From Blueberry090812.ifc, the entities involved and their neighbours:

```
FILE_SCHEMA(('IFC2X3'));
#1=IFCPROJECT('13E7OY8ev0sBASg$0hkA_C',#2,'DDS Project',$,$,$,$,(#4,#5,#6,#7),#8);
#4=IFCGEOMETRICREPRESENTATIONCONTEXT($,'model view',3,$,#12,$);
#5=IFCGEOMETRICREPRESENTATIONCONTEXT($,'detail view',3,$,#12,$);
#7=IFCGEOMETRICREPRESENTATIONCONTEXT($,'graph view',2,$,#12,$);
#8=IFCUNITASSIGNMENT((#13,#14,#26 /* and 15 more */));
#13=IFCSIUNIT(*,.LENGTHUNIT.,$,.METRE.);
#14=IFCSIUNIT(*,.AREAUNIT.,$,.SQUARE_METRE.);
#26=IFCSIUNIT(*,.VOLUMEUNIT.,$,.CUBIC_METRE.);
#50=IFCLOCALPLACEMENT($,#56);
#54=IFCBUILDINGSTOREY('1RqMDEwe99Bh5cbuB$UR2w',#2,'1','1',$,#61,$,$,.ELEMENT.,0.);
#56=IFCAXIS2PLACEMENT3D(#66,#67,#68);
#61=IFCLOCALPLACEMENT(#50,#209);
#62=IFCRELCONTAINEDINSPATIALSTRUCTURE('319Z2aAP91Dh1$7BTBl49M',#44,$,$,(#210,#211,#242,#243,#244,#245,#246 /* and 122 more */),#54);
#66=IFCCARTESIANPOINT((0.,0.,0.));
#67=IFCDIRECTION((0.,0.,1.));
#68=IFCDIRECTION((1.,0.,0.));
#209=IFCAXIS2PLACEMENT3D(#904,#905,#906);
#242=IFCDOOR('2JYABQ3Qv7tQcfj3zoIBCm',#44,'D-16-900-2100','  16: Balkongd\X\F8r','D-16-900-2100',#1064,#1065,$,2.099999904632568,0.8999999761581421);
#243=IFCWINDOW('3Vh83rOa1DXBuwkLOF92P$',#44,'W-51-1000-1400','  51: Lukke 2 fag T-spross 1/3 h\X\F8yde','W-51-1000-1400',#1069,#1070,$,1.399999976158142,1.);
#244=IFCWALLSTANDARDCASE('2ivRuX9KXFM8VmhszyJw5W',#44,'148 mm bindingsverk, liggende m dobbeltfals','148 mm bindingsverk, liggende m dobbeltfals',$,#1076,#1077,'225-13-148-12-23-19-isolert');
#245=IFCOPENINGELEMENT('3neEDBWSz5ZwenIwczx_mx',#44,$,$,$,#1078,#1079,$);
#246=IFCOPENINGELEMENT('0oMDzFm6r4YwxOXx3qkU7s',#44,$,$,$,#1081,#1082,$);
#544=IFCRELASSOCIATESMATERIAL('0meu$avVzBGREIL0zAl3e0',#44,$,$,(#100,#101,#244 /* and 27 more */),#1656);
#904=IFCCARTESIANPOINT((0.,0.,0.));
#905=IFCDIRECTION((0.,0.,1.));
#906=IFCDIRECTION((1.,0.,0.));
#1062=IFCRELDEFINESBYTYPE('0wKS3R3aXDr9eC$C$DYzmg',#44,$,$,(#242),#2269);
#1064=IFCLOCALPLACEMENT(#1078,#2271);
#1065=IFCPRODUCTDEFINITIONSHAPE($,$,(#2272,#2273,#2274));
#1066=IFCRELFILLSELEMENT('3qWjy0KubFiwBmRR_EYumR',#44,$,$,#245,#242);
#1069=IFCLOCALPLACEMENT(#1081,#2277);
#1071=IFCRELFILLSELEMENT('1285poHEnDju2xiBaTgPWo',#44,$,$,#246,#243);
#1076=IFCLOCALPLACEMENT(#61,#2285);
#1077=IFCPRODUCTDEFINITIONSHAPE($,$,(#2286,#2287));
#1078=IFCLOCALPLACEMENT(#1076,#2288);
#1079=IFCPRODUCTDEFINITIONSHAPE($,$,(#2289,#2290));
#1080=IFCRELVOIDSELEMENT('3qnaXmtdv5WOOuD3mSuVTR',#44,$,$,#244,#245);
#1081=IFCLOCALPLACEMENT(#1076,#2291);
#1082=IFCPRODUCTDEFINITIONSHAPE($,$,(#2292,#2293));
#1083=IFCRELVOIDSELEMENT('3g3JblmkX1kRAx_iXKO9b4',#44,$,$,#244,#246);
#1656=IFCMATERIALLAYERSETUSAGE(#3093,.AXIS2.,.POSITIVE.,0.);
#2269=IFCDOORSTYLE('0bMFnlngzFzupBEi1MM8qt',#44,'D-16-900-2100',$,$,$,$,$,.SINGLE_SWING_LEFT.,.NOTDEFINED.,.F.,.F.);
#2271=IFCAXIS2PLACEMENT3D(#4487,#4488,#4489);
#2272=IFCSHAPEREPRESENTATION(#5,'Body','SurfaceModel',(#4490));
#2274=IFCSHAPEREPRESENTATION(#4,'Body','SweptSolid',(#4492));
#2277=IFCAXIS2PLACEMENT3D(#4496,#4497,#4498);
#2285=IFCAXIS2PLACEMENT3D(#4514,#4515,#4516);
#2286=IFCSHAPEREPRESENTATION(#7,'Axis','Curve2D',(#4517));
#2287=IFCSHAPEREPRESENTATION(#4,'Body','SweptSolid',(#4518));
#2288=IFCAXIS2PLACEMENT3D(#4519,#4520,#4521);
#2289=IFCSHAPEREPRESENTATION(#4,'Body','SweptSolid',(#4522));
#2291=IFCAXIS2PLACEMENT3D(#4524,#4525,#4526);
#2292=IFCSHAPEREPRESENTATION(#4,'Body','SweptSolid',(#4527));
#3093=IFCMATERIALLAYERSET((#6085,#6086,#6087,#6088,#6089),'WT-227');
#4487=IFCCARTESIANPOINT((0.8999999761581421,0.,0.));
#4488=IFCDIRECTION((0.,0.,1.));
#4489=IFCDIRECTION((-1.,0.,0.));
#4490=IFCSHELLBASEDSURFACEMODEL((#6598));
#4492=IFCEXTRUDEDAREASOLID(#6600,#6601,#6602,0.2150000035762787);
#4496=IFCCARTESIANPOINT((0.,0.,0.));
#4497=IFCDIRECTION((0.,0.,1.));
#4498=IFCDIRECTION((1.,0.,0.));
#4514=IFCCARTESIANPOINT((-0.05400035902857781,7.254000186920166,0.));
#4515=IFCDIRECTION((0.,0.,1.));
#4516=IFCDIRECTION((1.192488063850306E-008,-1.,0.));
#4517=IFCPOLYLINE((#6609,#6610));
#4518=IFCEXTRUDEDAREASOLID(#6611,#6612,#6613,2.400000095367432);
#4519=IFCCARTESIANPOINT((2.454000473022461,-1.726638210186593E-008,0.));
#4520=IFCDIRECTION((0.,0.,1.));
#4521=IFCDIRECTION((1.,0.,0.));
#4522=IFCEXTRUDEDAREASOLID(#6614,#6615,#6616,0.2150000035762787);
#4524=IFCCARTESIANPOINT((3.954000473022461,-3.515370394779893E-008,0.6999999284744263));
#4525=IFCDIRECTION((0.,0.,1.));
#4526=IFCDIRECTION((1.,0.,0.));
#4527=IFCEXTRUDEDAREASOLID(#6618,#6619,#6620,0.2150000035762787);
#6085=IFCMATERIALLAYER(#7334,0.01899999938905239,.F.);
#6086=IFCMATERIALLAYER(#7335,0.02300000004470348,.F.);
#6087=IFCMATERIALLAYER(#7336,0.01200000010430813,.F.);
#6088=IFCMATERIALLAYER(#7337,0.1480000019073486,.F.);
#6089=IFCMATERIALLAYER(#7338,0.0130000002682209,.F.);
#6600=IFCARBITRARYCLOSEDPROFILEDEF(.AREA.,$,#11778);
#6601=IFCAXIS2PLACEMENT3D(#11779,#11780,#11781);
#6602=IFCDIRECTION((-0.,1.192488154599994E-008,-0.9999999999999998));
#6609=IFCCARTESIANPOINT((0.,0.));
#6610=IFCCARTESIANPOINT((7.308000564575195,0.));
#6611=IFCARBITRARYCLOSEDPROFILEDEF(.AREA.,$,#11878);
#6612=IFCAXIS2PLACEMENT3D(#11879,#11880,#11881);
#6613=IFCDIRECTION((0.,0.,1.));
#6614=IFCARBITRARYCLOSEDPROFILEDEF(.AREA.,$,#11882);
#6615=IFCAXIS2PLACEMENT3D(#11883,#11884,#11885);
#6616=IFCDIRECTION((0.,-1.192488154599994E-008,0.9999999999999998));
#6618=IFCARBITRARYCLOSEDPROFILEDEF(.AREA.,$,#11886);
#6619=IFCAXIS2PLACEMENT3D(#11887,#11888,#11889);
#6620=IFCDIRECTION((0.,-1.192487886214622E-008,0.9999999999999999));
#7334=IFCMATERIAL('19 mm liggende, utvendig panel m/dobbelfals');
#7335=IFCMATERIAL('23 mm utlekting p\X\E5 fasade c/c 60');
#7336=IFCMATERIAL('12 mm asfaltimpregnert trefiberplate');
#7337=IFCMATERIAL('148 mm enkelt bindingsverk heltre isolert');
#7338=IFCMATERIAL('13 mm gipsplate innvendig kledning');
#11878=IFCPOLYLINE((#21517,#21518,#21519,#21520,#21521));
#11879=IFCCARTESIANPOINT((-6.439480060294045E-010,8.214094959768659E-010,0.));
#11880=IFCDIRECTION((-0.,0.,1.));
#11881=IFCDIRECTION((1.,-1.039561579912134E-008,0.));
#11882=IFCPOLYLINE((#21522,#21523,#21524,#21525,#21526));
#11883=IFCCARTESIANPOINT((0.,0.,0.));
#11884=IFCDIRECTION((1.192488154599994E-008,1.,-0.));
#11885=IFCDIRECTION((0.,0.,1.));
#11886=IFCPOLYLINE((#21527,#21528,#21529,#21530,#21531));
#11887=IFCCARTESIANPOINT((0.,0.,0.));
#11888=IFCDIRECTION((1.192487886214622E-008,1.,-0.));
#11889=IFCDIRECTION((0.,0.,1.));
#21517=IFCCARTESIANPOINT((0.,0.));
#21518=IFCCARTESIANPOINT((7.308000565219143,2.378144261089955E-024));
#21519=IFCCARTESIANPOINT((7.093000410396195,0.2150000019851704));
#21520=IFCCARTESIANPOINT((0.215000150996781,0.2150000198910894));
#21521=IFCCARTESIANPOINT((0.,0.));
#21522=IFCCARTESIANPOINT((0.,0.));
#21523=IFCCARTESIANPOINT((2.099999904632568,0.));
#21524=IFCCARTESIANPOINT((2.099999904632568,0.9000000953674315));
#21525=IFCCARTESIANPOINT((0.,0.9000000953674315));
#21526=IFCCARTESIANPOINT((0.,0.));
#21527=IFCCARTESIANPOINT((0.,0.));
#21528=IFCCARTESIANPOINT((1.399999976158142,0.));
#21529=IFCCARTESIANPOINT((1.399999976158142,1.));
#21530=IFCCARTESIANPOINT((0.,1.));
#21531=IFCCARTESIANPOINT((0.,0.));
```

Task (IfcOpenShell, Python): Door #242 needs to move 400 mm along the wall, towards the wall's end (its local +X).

```python
import ifcopenshell
import ifcopenshell.api.geometry
import ifcopenshell.util.placement
import ifcopenshell.util.unit

model = ifcopenshell.open("Blueberry090812.ifc")
unit_scale = ifcopenshell.util.unit.calculate_unit_scale(model)

door = model.by_guid("2JYABQ3Qv7tQcfj3zoIBCm")
opening = door.FillsVoids[0].RelatingOpeningElement
wall = opening.VoidsElements[0].RelatingBuildingElement

wall_matrix = ifcopenshell.util.placement.get_local_placement(wall.ObjectPlacement)
shift = wall_matrix[:3, 0] * 0.4 / unit_scale
before = ifcopenshell.util.placement.get_local_placement(door.ObjectPlacement)[:3, 3].copy()

# The door is placed relative to its opening, so it follows when the opening moves.
matrix = ifcopenshell.util.placement.get_local_placement(opening.ObjectPlacement)
matrix[:3, 3] += shift
ifcopenshell.api.geometry.edit_object_placement(
    model, product=opening, matrix=matrix, is_si=False, should_transform_children=True
)

after = ifcopenshell.util.placement.get_local_placement(door.ObjectPlacement)[:3, 3]
print("door moved by", (after - before).round(3) + 0.0)

model.write("Blueberry090812_rev.ifc")
```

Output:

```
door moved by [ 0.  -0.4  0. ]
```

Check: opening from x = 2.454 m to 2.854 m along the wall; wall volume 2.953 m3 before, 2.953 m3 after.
